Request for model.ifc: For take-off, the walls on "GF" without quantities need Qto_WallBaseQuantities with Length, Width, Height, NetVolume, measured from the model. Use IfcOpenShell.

First a look at what the model holds.

```python
import ifcopenshell
import ifcopenshell.util.element
import ifcopenshell.util.unit

model = ifcopenshell.open("model.ifc")
print(model.schema)
for unit_type in ("LENGTHUNIT", "AREAUNIT", "VOLUMEUNIT"):
    print(unit_type, ifcopenshell.util.unit.calculate_unit_scale(model, unit_type))
storey = next(s for s in model.by_type("IfcBuildingStorey") if s.Name == "GF")
walls = [e for e in ifcopenshell.util.element.get_decomposition(storey) if e.is_a("IfcWall")]
for e in sorted(walls, key=lambda e: e.id()):
    print(e.id(), e.is_a(), e.Name, list(ifcopenshell.util.element.get_psets(e, qtos_only=True)), sep=" | ")
```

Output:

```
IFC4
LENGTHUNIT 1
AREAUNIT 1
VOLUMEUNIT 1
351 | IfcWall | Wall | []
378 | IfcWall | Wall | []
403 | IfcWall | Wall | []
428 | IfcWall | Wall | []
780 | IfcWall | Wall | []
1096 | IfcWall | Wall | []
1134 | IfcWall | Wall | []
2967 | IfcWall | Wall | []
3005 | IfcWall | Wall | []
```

```python
import ifcopenshell
import ifcopenshell.api.pset
import ifcopenshell.geom
import ifcopenshell.util.element
import ifcopenshell.util.shape
import ifcopenshell.util.unit

model = ifcopenshell.open("model.ifc")
unit_scale = ifcopenshell.util.unit.calculate_unit_scale(model)
volume_scale = ifcopenshell.util.unit.calculate_unit_scale(model, "VOLUMEUNIT")
settings = ifcopenshell.geom.settings()

storey = next(s for s in model.by_type("IfcBuildingStorey") if s.Name == "GF")
walls = [e for e in ifcopenshell.util.element.get_decomposition(storey) if e.is_a("IfcWall")]

for e in sorted(walls, key=lambda e: e.id()):
    if ifcopenshell.util.element.get_psets(e, qtos_only=True, should_inherit=False):
        continue
    # Geometry comes back in metres, in the element's own axes.
    shape = ifcopenshell.geom.create_shape(settings, e)
    values = {
        "Length": ifcopenshell.util.shape.get_x(shape.geometry) / unit_scale,
        "Width": ifcopenshell.util.shape.get_y(shape.geometry) / unit_scale,
        "Height": ifcopenshell.util.shape.get_z(shape.geometry) / unit_scale,
        "NetVolume": ifcopenshell.util.shape.get_volume(shape.geometry) / volume_scale,
    }
    qto = ifcopenshell.api.pset.add_qto(model, product=e, name="Qto_WallBaseQuantities")
    ifcopenshell.api.pset.edit_qto(model, qto=qto, properties=values)
    print(e.id(), {k: round(v, 3) for k, v in values.items()})

model.write("model-out.ifc")
```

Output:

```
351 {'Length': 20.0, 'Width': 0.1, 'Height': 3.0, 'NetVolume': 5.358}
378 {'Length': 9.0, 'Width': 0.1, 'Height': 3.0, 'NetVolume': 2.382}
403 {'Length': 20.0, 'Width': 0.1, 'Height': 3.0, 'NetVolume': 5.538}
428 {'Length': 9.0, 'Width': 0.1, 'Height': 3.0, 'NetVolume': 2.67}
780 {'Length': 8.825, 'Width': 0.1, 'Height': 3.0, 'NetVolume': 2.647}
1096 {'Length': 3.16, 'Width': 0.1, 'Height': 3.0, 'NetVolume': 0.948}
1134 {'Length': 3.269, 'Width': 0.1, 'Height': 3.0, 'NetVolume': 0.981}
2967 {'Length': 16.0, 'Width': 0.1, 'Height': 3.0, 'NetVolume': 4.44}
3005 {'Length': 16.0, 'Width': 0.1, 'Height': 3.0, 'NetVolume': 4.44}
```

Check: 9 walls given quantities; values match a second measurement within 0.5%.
